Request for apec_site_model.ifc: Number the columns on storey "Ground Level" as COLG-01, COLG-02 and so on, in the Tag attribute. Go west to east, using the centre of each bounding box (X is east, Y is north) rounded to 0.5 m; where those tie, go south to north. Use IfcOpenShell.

First a look at what the model holds.

```python
import ifcopenshell
import ifcopenshell.util.element
import ifcopenshell.util.placement

model = ifcopenshell.open("apec_site_model.ifc")
print(model.schema)
storey = next(s for s in model.by_type("IfcBuildingStorey") if s.Name == "Ground Level")
columns = [e for e in ifcopenshell.util.element.get_decomposition(storey) if e.is_a("IfcColumn")]
for e in sorted(columns, key=lambda e: e.id()):
    origin = ifcopenshell.util.placement.get_local_placement(e.ObjectPlacement)[:3, 3]
    print(e.id(), e.Tag, e.Name, origin.round(2) + 0.0, sep=" | ")
```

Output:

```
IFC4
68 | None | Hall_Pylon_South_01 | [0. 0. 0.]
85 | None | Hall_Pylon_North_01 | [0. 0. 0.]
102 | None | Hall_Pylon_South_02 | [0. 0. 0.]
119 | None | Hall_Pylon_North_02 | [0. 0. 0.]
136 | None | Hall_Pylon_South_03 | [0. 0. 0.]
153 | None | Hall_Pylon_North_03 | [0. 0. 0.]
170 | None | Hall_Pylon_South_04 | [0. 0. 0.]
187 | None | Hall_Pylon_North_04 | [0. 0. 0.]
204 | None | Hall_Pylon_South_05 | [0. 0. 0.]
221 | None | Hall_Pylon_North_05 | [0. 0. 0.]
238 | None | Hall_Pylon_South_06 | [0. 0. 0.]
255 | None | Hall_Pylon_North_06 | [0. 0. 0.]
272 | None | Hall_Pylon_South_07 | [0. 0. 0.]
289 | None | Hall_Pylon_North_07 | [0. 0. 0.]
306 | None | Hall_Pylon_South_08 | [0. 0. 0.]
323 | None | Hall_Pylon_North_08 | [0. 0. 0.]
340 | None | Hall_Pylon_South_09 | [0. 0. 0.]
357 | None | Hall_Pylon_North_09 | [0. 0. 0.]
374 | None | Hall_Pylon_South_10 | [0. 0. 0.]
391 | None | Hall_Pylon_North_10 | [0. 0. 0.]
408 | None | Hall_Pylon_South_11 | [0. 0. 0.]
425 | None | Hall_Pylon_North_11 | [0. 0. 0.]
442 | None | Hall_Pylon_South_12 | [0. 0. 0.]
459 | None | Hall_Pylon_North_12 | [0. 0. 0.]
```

```python
import ifcopenshell
import ifcopenshell.geom
import ifcopenshell.util.element
import ifcopenshell.util.shape

model = ifcopenshell.open("apec_site_model.ifc")
settings = ifcopenshell.geom.settings()
settings.set("use-world-coords", True)


def centre(element):
    shape = ifcopenshell.geom.create_shape(settings, element)
    return ifcopenshell.util.shape.get_bbox_centroid(shape.geometry)


storey = next(s for s in model.by_type("IfcBuildingStorey") if s.Name == "Ground Level")
columns = [e for e in ifcopenshell.util.element.get_decomposition(storey) if e.is_a("IfcColumn")]

# Insertion points can sit at a corner or the storey origin, so sort by the geometry (in metres).
centres = {e: centre(e) for e in columns}
columns.sort(key=lambda e: (round(centres[e][0] / 0.5), centres[e][1]))

for i, e in enumerate(columns, start=1):
    number = f"COLG-{i:02d}"
    e.Tag = number
    print(e.id(), number)

model.write("apec_site_model-out.ifc")
```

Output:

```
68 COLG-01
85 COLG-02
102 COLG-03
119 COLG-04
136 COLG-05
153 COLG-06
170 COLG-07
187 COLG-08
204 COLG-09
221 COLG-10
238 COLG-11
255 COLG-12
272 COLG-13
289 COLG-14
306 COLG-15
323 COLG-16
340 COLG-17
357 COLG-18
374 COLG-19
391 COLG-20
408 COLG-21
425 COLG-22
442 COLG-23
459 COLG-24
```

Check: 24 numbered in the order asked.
